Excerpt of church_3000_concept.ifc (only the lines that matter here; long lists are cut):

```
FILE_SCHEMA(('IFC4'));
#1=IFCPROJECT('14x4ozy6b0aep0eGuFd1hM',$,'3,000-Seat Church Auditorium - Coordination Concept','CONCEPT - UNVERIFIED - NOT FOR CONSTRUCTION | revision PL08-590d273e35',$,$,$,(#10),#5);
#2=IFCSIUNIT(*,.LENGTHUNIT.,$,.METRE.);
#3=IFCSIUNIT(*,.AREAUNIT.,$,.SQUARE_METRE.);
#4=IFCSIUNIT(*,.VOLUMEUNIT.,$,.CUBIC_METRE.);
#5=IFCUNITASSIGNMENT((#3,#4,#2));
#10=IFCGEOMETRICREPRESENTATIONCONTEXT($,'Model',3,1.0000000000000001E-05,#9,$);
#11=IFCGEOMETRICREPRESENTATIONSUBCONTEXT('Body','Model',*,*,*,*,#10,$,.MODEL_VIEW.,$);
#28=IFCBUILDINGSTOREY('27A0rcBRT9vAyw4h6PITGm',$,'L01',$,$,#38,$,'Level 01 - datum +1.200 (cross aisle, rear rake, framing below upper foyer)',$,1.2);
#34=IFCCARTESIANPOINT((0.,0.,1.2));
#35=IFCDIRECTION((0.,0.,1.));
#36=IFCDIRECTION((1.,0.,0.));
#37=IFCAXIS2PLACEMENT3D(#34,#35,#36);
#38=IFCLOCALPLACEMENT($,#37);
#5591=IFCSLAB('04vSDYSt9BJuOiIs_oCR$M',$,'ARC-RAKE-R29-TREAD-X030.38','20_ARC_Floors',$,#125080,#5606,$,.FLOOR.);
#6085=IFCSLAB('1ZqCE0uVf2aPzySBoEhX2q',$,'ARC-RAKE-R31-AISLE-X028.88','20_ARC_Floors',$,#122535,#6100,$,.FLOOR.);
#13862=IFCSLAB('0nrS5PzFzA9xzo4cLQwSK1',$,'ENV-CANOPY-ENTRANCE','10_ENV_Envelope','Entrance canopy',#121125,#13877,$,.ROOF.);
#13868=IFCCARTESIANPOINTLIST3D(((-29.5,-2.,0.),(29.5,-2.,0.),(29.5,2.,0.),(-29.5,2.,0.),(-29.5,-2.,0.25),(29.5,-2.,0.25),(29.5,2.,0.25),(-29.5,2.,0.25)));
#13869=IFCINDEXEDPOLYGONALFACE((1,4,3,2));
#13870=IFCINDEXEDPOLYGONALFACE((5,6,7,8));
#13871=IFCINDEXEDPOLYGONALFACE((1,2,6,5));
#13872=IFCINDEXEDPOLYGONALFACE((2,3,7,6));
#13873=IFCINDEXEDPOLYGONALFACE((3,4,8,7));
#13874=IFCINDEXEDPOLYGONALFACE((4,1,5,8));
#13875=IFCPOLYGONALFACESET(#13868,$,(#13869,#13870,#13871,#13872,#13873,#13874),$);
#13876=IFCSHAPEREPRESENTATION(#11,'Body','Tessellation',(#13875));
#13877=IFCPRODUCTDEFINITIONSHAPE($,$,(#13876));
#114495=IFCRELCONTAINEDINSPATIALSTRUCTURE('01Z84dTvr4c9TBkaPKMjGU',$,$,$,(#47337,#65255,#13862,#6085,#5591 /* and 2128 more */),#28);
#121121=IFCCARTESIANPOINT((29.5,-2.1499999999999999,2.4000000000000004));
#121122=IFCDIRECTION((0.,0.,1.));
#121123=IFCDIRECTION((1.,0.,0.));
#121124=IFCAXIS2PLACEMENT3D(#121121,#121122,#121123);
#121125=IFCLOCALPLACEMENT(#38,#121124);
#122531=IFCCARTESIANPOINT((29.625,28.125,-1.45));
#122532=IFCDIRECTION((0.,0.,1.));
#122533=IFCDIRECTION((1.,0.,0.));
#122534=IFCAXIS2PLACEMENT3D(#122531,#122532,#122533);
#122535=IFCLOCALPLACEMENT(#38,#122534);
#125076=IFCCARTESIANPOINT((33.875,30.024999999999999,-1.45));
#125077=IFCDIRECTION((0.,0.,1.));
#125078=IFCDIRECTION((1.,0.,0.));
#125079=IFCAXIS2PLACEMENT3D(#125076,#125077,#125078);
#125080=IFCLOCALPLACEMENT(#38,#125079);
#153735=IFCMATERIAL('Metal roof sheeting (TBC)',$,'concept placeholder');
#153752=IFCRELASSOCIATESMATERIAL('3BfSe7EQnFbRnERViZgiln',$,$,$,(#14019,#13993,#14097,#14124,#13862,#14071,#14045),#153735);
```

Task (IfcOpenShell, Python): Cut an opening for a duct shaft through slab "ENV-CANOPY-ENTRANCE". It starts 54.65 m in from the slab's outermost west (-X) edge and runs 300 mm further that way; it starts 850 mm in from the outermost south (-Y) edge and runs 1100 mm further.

```python
import numpy as np
import ifcopenshell
import ifcopenshell.api.feature
import ifcopenshell.api.geometry
import ifcopenshell.api.root
import ifcopenshell.geom
import ifcopenshell.util.placement
import ifcopenshell.util.representation
import ifcopenshell.util.shape
import ifcopenshell.util.unit

model = ifcopenshell.open("church_3000_concept.ifc")
unit_scale = ifcopenshell.util.unit.calculate_unit_scale(model)
settings = ifcopenshell.geom.settings()


def volume(element):
    """Net volume in cubic metres, openings subtracted."""
    shape = ifcopenshell.geom.create_shape(settings, element)
    return ifcopenshell.util.shape.get_volume(shape.geometry)


slab = model.by_guid("0nrS5PzFzA9xzo4cLQwSK1")
before = volume(slab)

# Extent in the slab's own axes, in metres. The edges named are its -X and -Y sides.
slab_shape = ifcopenshell.geom.create_shape(settings, slab)
vertices = ifcopenshell.util.shape.get_vertices(slab_shape.geometry)
x_min, y_min, bottom = vertices.min(axis=0)
top = vertices[:, 2].max()

opening = ifcopenshell.api.root.create_entity(model, ifc_class="IfcOpeningElement", name="Duct shaft opening", predefined_type="OPENING")
context = ifcopenshell.util.representation.get_context(model, "Model", "Body", "MODEL_VIEW")
width, depth = 0.3, 1.1
outline = [(0.0, 0.0), (width, 0.0), (width, depth), (0.0, depth), (0.0, 0.0)]
# Overshoot both faces by 50 mm so the cut is clean.
shape = ifcopenshell.api.geometry.add_slab_representation(
    model, context=context, depth=top - bottom + 0.1, polyline=outline
)
ifcopenshell.api.geometry.assign_representation(model, product=opening, representation=shape)

matrix = ifcopenshell.util.placement.get_local_placement(slab.ObjectPlacement)
matrix[:, 3] = matrix @ np.append(np.array([x_min + 54.65, y_min + 0.85, bottom - 0.05]) / unit_scale, 1.0)
ifcopenshell.api.geometry.edit_object_placement(model, product=opening, matrix=matrix, is_si=False)
ifcopenshell.api.feature.add_feature(model, feature=opening, element=slab)

after = volume(slab)

print(f"slab volume {before:.3f} -> {after:.3f} m3")

model.write("church_3000_concept_v2.ifc")
```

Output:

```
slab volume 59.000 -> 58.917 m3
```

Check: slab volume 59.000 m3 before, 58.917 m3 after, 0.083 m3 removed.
